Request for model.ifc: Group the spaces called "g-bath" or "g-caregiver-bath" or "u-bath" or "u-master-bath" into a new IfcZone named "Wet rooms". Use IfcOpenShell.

First a look at what the model holds.

```python
import ifcopenshell

model = ifcopenshell.open("model.ifc")
print(model.schema)
seen = {}
for space in model.by_type("IfcSpace"):
    seen[space.LongName] = seen.get(space.LongName, 0) + 1
for name, count in sorted(seen.items(), key=str):
    print(count, "x", name)
print("zones:", [z.Name for z in model.by_type("IfcZone")][:20])
```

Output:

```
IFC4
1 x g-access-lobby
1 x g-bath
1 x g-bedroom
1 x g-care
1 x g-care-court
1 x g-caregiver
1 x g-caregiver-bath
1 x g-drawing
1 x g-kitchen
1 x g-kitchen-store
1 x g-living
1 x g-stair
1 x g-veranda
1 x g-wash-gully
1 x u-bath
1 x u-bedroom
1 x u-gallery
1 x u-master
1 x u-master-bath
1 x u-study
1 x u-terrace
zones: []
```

```python
import ifcopenshell
import ifcopenshell.api.group
import ifcopenshell.api.root

model = ifcopenshell.open("model.ifc")

names = {"g-bath", "g-caregiver-bath", "u-bath", "u-master-bath"}
spaces = [s for s in model.by_type("IfcSpace") if s.LongName in names]

zone = ifcopenshell.api.root.create_entity(model, ifc_class="IfcZone", name="Wet rooms")
ifcopenshell.api.group.assign_group(model, products=spaces, group=zone)
print(len(spaces), "spaces in", zone.Name)

model.write("model-out.ifc")
```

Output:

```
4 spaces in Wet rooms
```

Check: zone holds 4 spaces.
